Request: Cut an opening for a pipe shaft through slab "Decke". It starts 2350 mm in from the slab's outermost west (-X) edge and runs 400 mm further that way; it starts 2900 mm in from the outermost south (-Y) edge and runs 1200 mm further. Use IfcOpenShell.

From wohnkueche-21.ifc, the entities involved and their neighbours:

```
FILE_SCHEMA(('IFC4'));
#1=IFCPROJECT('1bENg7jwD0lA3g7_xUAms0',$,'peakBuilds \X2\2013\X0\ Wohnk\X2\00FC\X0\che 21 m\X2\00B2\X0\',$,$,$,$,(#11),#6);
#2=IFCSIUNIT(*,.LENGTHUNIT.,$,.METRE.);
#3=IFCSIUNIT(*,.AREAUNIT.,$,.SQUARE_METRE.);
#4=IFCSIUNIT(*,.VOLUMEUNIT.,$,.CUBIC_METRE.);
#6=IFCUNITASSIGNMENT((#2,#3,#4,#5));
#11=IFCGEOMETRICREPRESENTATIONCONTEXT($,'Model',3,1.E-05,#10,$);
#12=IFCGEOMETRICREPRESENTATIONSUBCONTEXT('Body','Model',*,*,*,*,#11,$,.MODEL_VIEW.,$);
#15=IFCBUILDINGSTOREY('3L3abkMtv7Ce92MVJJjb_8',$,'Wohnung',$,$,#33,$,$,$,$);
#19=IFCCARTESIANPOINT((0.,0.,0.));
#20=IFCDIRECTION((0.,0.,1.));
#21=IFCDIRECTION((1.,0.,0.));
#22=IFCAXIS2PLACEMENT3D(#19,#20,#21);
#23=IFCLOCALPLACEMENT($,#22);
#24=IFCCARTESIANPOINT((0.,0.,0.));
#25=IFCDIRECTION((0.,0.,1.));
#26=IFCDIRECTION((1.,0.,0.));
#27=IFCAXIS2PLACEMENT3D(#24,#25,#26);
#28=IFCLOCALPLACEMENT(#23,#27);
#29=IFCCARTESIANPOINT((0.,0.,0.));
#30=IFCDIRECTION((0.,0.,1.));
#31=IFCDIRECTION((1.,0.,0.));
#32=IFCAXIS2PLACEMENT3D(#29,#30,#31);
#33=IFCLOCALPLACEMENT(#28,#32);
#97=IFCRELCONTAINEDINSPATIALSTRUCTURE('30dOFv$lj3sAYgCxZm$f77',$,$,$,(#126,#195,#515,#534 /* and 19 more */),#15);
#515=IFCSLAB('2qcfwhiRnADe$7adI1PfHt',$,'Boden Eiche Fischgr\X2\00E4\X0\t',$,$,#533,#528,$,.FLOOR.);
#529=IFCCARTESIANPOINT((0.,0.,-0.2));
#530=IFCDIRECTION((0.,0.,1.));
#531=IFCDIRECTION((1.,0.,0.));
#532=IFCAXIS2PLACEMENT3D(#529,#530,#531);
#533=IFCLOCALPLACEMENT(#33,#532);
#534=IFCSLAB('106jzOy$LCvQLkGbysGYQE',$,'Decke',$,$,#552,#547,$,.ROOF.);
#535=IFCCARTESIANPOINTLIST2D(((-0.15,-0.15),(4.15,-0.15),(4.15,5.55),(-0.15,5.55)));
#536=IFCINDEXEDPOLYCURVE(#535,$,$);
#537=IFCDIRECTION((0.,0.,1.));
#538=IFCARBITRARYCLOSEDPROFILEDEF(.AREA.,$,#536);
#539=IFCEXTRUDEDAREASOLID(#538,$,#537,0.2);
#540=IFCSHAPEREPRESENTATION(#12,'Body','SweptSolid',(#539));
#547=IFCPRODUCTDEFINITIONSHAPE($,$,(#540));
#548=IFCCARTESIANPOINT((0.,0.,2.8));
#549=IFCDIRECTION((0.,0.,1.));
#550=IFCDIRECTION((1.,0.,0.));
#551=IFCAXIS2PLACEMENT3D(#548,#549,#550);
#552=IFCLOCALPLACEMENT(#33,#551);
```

```python
import numpy as np
import ifcopenshell
import ifcopenshell.api.feature
import ifcopenshell.api.geometry
import ifcopenshell.api.root
import ifcopenshell.geom
import ifcopenshell.util.placement
import ifcopenshell.util.representation
import ifcopenshell.util.shape
import ifcopenshell.util.unit

model = ifcopenshell.open("wohnkueche-21.ifc")
unit_scale = ifcopenshell.util.unit.calculate_unit_scale(model)
settings = ifcopenshell.geom.settings()


def volume(element):
    """Net volume in cubic metres, openings subtracted."""
    shape = ifcopenshell.geom.create_shape(settings, element)
    return ifcopenshell.util.shape.get_volume(shape.geometry)


slab = model.by_guid("106jzOy$LCvQLkGbysGYQE")
before = volume(slab)

# Extent in the slab's own axes, in metres. The edges named are its -X and -Y sides.
slab_shape = ifcopenshell.geom.create_shape(settings, slab)
vertices = ifcopenshell.util.shape.get_vertices(slab_shape.geometry)
x_min, y_min, bottom = vertices.min(axis=0)
top = vertices[:, 2].max()

opening = ifcopenshell.api.root.create_entity(model, ifc_class="IfcOpeningElement", name="Pipe shaft opening", predefined_type="OPENING")
context = ifcopenshell.util.representation.get_context(model, "Model", "Body", "MODEL_VIEW")
width, depth = 0.4, 1.2
outline = [(0.0, 0.0), (width, 0.0), (width, depth), (0.0, depth), (0.0, 0.0)]
# Overshoot both faces by 50 mm so the cut is clean.
shape = ifcopenshell.api.geometry.add_slab_representation(
    model, context=context, depth=top - bottom + 0.1, polyline=outline
)
ifcopenshell.api.geometry.assign_representation(model, product=opening, representation=shape)

matrix = ifcopenshell.util.placement.get_local_placement(slab.ObjectPlacement)
matrix[:, 3] = matrix @ np.append(np.array([x_min + 2.35, y_min + 2.9, bottom - 0.05]) / unit_scale, 1.0)
ifcopenshell.api.geometry.edit_object_placement(model, product=opening, matrix=matrix, is_si=False)
ifcopenshell.api.feature.add_feature(model, feature=opening, element=slab)

after = volume(slab)

print(f"slab volume {before:.3f} -> {after:.3f} m3")

model.write("wohnkueche-21-out.ifc")
```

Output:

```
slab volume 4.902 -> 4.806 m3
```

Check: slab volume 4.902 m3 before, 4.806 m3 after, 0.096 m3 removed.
